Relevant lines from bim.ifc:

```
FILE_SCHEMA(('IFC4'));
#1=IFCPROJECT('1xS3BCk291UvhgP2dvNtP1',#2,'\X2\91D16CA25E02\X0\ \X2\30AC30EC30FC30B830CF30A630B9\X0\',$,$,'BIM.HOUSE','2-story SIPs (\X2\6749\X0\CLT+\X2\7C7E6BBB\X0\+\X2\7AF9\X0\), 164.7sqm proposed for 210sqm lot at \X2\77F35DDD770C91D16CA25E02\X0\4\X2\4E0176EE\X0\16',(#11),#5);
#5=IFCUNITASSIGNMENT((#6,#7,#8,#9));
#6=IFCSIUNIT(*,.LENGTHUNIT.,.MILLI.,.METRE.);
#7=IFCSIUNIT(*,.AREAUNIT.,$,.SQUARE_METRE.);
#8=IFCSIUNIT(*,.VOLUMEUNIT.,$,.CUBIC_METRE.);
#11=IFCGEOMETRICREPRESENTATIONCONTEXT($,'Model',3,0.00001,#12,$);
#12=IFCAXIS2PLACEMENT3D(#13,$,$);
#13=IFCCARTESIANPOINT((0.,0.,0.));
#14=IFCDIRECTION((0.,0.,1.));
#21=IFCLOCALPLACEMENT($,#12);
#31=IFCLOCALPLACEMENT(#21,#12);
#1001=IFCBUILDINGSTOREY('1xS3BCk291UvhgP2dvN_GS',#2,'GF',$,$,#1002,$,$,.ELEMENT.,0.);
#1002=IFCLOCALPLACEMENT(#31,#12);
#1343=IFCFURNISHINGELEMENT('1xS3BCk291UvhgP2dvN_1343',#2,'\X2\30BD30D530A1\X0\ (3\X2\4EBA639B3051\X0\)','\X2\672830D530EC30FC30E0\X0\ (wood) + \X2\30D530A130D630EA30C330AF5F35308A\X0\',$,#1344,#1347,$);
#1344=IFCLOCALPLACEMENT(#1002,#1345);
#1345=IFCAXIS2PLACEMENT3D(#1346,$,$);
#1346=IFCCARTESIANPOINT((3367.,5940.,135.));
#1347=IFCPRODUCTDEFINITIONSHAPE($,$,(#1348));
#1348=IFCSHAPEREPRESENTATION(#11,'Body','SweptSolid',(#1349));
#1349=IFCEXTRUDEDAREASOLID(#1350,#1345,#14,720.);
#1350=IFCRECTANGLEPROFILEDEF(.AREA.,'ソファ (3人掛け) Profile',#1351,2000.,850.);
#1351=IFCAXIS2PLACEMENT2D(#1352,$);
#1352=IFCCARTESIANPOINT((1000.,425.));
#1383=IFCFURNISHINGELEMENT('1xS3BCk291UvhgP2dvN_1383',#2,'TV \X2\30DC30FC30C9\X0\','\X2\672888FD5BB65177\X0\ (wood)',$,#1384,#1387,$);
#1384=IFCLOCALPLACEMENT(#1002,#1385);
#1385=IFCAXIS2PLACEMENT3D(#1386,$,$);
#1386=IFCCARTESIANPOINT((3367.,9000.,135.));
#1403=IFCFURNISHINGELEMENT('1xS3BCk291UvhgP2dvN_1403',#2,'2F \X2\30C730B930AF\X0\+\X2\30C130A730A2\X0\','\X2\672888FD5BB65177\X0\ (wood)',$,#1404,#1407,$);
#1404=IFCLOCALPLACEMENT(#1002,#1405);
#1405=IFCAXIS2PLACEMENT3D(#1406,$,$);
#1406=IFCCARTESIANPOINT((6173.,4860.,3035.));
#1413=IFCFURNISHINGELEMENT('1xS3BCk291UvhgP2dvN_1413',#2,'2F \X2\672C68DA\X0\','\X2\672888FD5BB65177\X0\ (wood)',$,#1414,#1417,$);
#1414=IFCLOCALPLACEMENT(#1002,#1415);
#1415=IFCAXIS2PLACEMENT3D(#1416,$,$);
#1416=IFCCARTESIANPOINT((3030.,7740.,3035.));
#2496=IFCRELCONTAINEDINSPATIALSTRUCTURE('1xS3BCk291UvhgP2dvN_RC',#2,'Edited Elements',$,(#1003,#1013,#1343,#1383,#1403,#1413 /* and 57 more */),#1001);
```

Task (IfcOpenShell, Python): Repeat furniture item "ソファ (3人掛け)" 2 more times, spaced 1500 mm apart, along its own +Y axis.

```python
import ifcopenshell
import ifcopenshell.api.geometry
import ifcopenshell.api.root
import ifcopenshell.util.element
import ifcopenshell.util.placement

model = ifcopenshell.open("bim.ifc")


def reuse_history(source, copy):
    """copy_class also copies each property set's owner history, people and application; keep the originals."""
    for rel in copy.IsDefinedBy:
        if rel.is_a("IfcRelDefinesByProperties") and (history := rel.RelatingPropertyDefinition.OwnerHistory):
            rel.RelatingPropertyDefinition.OwnerHistory = source.OwnerHistory
            ifcopenshell.util.element.remove_deep2(model, history)


source = model.by_guid("1xS3BCk291UvhgP2dvN_1343")
base = ifcopenshell.util.placement.get_local_placement(source.ObjectPlacement)
step = base[:3, 1] * 1500.0

for i in range(1, 3):
    copy = ifcopenshell.api.root.copy_class(model, product=source)
    copy.Representation = ifcopenshell.util.element.copy_deep(
        model, source.Representation, exclude=["IfcGeometricRepresentationContext", "IfcRepresentationMap"]
    )
    reuse_history(source, copy)
    matrix = base.copy()
    matrix[:3, 3] += i * step
    print("added at", matrix[:3, 3].round(3) + 0.0)
    ifcopenshell.api.geometry.edit_object_placement(model, product=copy, matrix=matrix, is_si=False)

model.write("bim_v2.ifc")
```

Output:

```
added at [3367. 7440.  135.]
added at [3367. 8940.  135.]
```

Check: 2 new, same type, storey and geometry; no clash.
